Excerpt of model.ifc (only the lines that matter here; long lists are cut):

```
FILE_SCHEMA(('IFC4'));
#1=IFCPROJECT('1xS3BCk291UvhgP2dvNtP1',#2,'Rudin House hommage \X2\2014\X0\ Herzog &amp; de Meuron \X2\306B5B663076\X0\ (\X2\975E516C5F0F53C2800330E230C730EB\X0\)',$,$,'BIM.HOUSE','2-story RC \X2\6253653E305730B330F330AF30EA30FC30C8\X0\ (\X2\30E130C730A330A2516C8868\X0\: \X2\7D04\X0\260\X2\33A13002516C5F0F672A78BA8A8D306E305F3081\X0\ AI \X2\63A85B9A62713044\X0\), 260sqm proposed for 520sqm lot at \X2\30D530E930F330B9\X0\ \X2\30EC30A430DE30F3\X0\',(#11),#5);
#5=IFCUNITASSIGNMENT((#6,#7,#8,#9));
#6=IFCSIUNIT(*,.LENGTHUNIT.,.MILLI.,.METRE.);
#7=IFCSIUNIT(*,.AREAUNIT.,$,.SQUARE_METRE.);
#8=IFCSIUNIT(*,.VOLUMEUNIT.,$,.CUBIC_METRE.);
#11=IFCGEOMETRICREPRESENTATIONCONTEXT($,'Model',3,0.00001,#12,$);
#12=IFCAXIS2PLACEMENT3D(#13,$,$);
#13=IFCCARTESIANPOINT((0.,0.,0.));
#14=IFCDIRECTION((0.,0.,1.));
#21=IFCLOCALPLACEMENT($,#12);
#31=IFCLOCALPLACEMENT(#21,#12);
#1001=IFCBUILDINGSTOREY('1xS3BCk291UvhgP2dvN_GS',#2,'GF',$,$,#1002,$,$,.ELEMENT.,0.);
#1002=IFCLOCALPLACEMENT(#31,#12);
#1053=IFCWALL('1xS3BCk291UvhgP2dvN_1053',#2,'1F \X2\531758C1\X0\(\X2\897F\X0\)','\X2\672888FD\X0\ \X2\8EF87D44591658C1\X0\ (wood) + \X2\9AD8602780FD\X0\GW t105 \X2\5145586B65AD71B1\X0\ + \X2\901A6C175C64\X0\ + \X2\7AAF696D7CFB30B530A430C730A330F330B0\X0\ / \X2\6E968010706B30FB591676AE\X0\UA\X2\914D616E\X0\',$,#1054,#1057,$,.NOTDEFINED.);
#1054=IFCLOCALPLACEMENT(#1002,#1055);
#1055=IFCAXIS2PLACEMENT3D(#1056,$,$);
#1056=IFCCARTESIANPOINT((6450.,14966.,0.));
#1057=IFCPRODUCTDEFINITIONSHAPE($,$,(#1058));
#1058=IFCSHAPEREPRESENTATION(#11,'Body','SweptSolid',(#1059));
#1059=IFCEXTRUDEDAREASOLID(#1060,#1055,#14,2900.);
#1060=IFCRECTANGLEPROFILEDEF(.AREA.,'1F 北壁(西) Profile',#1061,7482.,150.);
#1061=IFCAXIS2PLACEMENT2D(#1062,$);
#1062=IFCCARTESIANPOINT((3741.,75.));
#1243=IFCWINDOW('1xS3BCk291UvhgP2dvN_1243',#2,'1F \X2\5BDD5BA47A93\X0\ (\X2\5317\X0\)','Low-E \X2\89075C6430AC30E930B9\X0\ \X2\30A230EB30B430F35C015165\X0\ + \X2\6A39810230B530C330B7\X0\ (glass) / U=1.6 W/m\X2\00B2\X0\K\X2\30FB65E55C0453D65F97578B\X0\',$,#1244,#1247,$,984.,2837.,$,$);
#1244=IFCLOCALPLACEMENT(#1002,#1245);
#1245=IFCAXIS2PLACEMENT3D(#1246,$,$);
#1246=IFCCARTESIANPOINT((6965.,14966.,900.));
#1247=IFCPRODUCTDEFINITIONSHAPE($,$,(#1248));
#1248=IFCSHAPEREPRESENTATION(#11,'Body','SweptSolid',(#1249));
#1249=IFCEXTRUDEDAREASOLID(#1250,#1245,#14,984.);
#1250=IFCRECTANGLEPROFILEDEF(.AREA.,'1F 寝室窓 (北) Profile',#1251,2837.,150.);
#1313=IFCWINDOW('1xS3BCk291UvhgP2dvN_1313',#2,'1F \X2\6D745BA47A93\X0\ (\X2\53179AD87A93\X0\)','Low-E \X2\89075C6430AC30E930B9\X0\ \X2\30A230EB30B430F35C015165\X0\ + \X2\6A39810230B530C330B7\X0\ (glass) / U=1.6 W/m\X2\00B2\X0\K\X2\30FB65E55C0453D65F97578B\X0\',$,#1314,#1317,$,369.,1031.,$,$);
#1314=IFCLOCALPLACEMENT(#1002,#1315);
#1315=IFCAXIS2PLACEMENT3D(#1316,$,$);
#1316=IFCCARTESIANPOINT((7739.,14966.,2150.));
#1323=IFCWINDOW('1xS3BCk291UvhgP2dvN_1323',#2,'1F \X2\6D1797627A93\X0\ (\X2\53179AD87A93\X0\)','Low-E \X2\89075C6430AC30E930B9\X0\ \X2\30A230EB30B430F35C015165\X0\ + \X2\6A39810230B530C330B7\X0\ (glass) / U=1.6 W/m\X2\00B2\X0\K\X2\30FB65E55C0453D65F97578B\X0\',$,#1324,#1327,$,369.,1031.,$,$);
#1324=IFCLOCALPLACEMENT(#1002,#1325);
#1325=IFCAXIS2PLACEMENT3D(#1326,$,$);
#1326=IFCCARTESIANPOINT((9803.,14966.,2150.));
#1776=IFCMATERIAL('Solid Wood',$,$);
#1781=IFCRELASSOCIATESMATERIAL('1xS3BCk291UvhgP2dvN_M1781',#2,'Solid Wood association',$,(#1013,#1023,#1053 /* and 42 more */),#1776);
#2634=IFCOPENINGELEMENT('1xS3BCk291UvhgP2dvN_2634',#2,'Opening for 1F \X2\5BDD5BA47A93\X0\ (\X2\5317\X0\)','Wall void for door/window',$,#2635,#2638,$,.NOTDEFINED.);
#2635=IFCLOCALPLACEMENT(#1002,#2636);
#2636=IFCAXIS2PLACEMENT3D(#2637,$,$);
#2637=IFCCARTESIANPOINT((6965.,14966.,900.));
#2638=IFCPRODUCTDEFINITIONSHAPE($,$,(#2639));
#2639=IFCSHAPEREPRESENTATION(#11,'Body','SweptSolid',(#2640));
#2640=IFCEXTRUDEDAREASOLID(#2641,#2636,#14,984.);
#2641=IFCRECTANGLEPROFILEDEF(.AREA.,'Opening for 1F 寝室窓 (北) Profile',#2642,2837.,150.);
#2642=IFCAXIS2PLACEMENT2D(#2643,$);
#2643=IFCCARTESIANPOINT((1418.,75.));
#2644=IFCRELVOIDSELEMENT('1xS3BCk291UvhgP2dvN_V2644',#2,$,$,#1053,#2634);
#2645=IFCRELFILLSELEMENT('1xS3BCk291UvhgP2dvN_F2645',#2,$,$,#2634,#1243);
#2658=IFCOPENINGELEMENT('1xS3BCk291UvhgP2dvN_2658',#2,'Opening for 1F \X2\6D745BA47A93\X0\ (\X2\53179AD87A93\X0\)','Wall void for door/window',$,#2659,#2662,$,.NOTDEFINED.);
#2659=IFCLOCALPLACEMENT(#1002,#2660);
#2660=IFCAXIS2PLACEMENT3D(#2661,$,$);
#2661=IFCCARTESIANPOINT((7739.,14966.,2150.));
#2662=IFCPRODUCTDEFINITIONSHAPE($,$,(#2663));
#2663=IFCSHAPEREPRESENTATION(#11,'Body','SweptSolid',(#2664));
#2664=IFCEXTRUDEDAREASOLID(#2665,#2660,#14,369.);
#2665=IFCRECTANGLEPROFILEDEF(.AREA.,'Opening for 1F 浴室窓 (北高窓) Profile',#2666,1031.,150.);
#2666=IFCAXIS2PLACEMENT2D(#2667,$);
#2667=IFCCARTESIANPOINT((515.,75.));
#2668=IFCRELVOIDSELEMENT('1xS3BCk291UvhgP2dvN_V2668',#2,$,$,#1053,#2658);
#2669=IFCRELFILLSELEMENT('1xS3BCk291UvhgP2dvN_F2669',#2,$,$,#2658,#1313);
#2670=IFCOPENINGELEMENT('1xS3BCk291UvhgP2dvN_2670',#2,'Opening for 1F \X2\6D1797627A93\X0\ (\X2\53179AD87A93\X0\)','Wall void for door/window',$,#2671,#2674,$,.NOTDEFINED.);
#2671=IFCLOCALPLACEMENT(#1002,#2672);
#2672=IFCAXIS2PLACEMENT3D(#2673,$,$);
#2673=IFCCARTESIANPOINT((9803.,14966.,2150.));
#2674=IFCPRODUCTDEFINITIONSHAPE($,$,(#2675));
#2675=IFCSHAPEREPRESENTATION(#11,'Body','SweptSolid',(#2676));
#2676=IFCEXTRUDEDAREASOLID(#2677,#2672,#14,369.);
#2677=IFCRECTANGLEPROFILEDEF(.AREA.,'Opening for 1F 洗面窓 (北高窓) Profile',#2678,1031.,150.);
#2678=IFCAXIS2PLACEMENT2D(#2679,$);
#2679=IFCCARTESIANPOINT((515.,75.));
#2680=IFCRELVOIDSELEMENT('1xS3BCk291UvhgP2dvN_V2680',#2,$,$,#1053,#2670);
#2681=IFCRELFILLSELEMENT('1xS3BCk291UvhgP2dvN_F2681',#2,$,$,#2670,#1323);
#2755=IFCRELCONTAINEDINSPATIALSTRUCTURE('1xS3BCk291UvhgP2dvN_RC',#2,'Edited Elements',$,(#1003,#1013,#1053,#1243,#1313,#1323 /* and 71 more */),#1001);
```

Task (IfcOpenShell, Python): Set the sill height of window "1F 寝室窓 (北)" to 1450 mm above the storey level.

```python
import numpy as np
import ifcopenshell
import ifcopenshell.api.geometry
import ifcopenshell.geom
import ifcopenshell.util.element
import ifcopenshell.util.placement
import ifcopenshell.util.shape
import ifcopenshell.util.unit

model = ifcopenshell.open("model.ifc")
unit_scale = ifcopenshell.util.unit.calculate_unit_scale(model)

window = model.by_guid("1xS3BCk291UvhgP2dvN_1243")
opening = window.FillsVoids[0].RelatingOpeningElement
storey = ifcopenshell.util.element.get_container(window, ifc_class="IfcBuildingStorey")
level = ifcopenshell.util.placement.get_local_placement(storey.ObjectPlacement)[2, 3]

# The opening's origin need not be at the sill, so measure its lowest point.
shape = ifcopenshell.geom.create_shape(ifcopenshell.geom.settings(), opening)
bottom = ifcopenshell.util.shape.get_shape_bottom_elevation(shape, shape.geometry) / unit_scale
dz = level + 1.45 / unit_scale - bottom

shift = np.array([0.0, 0.0, dz])
# The window is not placed relative to its opening, so move both.
for product in (opening, window):
    matrix = ifcopenshell.util.placement.get_local_placement(product.ObjectPlacement)
    matrix[:3, 3] += shift
    ifcopenshell.api.geometry.edit_object_placement(model, product=product, matrix=matrix, is_si=False)

print(f"moved by {dz * unit_scale:+.3f} m")

model.write("model_v2.ifc")
```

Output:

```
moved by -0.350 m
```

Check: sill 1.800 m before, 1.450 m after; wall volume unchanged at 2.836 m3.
